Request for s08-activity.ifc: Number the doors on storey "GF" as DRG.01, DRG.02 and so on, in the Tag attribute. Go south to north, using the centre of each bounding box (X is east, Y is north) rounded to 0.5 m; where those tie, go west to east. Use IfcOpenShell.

First a look at what the model holds.

```python
import ifcopenshell
import ifcopenshell.util.element
import ifcopenshell.util.placement

model = ifcopenshell.open("s08-activity.ifc")
print(model.schema)
storey = next(s for s in model.by_type("IfcBuildingStorey") if s.Name == "GF")
doors = [e for e in ifcopenshell.util.element.get_decomposition(storey) if e.is_a("IfcDoor")]
for e in sorted(doors, key=lambda e: e.id()):
    origin = ifcopenshell.util.placement.get_local_placement(e.ObjectPlacement)[:3, 3]
    print(e.id(), e.Tag, e.Name, origin.round(2) + 0.0, sep=" | ")
```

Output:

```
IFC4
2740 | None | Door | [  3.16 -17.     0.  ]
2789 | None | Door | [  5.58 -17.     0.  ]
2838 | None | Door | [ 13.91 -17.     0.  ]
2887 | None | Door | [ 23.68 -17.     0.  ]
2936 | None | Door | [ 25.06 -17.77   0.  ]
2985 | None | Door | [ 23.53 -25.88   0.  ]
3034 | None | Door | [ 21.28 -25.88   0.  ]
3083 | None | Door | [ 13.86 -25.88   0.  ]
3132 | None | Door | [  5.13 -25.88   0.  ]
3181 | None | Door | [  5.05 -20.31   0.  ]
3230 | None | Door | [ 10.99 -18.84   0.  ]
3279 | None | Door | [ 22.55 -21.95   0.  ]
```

```python
import ifcopenshell
import ifcopenshell.geom
import ifcopenshell.util.element
import ifcopenshell.util.shape

model = ifcopenshell.open("s08-activity.ifc")
settings = ifcopenshell.geom.settings()
settings.set("use-world-coords", True)


def centre(element):
    shape = ifcopenshell.geom.create_shape(settings, element)
    return ifcopenshell.util.shape.get_bbox_centroid(shape.geometry)


storey = next(s for s in model.by_type("IfcBuildingStorey") if s.Name == "GF")
doors = [e for e in ifcopenshell.util.element.get_decomposition(storey) if e.is_a("IfcDoor")]

# Insertion points can sit at a corner or the storey origin, so sort by the geometry (in metres).
centres = {e: centre(e) for e in doors}
doors.sort(key=lambda e: (round(centres[e][1] / 0.5), centres[e][0]))

for i, e in enumerate(doors, start=1):
    number = f"DRG.{i:02d}"
    e.Tag = number
    print(e.id(), number)

model.write("s08-activity_edited.ifc")
```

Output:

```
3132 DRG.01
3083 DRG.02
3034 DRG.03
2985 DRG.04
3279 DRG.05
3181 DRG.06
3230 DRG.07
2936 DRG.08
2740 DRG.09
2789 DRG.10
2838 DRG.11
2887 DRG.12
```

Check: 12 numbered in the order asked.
